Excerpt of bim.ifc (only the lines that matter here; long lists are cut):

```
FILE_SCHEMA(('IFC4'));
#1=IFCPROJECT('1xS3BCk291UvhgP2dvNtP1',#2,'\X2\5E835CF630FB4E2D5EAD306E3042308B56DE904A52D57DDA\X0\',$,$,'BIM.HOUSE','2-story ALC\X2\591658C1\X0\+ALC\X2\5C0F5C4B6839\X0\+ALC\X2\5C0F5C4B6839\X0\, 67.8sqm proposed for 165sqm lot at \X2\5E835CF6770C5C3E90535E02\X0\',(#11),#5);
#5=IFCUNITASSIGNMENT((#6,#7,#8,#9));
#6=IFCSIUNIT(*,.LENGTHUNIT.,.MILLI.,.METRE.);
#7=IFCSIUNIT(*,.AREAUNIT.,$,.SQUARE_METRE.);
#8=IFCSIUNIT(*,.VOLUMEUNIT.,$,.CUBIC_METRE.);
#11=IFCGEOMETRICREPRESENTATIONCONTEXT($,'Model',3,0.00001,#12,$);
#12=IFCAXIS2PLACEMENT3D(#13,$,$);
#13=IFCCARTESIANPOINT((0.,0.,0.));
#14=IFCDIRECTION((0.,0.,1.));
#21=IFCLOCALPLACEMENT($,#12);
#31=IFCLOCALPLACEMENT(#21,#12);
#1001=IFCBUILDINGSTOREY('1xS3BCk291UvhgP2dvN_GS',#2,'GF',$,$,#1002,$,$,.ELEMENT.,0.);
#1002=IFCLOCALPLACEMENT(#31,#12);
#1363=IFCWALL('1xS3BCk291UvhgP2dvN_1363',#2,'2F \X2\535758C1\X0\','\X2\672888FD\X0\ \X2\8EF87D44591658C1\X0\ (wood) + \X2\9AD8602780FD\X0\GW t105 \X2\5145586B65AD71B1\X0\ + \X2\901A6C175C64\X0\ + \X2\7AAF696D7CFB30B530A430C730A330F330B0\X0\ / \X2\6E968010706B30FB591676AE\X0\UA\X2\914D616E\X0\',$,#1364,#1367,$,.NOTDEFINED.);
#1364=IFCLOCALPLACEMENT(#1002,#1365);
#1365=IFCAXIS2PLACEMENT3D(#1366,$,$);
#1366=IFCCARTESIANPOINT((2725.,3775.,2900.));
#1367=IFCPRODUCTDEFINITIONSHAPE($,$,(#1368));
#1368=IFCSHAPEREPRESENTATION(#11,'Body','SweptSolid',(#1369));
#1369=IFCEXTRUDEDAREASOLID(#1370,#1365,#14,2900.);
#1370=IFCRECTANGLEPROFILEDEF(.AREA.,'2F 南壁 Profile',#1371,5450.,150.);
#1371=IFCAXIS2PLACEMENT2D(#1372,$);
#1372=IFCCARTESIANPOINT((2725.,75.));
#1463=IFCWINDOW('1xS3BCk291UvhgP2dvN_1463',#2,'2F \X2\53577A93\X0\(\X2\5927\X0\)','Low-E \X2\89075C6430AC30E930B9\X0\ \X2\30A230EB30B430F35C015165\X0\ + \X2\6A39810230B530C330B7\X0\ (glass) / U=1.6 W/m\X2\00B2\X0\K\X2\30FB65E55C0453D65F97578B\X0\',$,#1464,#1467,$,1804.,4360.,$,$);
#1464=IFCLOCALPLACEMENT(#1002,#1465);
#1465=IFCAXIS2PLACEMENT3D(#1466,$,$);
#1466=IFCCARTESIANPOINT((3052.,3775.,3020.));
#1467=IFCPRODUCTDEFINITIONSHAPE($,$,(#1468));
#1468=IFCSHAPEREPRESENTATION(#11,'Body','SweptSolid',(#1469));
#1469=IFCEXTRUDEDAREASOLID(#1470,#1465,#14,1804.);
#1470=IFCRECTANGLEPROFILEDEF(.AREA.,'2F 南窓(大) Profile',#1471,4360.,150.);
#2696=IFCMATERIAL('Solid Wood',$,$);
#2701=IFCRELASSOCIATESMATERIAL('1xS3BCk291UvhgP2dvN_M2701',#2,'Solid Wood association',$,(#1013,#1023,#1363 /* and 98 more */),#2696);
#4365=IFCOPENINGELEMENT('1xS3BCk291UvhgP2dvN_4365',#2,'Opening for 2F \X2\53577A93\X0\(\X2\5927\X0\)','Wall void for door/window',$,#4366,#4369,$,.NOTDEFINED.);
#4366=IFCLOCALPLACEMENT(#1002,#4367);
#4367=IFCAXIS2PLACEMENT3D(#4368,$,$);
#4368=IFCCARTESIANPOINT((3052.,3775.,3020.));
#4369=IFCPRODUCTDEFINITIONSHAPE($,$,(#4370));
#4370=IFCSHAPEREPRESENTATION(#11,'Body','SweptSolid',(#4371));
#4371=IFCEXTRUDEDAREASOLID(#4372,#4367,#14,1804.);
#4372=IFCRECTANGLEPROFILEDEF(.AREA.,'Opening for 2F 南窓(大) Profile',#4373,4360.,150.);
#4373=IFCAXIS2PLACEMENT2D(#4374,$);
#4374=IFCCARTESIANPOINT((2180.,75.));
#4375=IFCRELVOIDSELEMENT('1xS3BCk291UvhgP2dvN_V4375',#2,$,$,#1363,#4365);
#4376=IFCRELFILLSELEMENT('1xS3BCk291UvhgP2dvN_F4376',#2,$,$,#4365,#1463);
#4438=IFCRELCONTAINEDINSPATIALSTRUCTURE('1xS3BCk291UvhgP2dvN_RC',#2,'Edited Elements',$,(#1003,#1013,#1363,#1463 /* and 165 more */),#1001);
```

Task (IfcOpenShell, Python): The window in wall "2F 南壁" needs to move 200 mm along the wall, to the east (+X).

```python
import ifcopenshell
import ifcopenshell.api.geometry
import ifcopenshell.util.placement
import ifcopenshell.util.unit

model = ifcopenshell.open("bim.ifc")
unit_scale = ifcopenshell.util.unit.calculate_unit_scale(model)

window = model.by_guid("1xS3BCk291UvhgP2dvN_1463")
opening = window.FillsVoids[0].RelatingOpeningElement
wall = opening.VoidsElements[0].RelatingBuildingElement

wall_matrix = ifcopenshell.util.placement.get_local_placement(wall.ObjectPlacement)
shift = wall_matrix[:3, 0] * 0.2 / unit_scale
before = ifcopenshell.util.placement.get_local_placement(window.ObjectPlacement)[:3, 3].copy()

# The window is not placed relative to its opening, so move both.
for product in (opening, window):
    matrix = ifcopenshell.util.placement.get_local_placement(product.ObjectPlacement)
    matrix[:3, 3] += shift
    ifcopenshell.api.geometry.edit_object_placement(model, product=product, matrix=matrix, is_si=False)

after = ifcopenshell.util.placement.get_local_placement(window.ObjectPlacement)[:3, 3]
print("window moved by", (after - before).round(3) + 0.0)

model.write("bim_rev.ifc")
```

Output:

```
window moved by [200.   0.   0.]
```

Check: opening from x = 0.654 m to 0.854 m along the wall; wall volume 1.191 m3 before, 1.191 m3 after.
